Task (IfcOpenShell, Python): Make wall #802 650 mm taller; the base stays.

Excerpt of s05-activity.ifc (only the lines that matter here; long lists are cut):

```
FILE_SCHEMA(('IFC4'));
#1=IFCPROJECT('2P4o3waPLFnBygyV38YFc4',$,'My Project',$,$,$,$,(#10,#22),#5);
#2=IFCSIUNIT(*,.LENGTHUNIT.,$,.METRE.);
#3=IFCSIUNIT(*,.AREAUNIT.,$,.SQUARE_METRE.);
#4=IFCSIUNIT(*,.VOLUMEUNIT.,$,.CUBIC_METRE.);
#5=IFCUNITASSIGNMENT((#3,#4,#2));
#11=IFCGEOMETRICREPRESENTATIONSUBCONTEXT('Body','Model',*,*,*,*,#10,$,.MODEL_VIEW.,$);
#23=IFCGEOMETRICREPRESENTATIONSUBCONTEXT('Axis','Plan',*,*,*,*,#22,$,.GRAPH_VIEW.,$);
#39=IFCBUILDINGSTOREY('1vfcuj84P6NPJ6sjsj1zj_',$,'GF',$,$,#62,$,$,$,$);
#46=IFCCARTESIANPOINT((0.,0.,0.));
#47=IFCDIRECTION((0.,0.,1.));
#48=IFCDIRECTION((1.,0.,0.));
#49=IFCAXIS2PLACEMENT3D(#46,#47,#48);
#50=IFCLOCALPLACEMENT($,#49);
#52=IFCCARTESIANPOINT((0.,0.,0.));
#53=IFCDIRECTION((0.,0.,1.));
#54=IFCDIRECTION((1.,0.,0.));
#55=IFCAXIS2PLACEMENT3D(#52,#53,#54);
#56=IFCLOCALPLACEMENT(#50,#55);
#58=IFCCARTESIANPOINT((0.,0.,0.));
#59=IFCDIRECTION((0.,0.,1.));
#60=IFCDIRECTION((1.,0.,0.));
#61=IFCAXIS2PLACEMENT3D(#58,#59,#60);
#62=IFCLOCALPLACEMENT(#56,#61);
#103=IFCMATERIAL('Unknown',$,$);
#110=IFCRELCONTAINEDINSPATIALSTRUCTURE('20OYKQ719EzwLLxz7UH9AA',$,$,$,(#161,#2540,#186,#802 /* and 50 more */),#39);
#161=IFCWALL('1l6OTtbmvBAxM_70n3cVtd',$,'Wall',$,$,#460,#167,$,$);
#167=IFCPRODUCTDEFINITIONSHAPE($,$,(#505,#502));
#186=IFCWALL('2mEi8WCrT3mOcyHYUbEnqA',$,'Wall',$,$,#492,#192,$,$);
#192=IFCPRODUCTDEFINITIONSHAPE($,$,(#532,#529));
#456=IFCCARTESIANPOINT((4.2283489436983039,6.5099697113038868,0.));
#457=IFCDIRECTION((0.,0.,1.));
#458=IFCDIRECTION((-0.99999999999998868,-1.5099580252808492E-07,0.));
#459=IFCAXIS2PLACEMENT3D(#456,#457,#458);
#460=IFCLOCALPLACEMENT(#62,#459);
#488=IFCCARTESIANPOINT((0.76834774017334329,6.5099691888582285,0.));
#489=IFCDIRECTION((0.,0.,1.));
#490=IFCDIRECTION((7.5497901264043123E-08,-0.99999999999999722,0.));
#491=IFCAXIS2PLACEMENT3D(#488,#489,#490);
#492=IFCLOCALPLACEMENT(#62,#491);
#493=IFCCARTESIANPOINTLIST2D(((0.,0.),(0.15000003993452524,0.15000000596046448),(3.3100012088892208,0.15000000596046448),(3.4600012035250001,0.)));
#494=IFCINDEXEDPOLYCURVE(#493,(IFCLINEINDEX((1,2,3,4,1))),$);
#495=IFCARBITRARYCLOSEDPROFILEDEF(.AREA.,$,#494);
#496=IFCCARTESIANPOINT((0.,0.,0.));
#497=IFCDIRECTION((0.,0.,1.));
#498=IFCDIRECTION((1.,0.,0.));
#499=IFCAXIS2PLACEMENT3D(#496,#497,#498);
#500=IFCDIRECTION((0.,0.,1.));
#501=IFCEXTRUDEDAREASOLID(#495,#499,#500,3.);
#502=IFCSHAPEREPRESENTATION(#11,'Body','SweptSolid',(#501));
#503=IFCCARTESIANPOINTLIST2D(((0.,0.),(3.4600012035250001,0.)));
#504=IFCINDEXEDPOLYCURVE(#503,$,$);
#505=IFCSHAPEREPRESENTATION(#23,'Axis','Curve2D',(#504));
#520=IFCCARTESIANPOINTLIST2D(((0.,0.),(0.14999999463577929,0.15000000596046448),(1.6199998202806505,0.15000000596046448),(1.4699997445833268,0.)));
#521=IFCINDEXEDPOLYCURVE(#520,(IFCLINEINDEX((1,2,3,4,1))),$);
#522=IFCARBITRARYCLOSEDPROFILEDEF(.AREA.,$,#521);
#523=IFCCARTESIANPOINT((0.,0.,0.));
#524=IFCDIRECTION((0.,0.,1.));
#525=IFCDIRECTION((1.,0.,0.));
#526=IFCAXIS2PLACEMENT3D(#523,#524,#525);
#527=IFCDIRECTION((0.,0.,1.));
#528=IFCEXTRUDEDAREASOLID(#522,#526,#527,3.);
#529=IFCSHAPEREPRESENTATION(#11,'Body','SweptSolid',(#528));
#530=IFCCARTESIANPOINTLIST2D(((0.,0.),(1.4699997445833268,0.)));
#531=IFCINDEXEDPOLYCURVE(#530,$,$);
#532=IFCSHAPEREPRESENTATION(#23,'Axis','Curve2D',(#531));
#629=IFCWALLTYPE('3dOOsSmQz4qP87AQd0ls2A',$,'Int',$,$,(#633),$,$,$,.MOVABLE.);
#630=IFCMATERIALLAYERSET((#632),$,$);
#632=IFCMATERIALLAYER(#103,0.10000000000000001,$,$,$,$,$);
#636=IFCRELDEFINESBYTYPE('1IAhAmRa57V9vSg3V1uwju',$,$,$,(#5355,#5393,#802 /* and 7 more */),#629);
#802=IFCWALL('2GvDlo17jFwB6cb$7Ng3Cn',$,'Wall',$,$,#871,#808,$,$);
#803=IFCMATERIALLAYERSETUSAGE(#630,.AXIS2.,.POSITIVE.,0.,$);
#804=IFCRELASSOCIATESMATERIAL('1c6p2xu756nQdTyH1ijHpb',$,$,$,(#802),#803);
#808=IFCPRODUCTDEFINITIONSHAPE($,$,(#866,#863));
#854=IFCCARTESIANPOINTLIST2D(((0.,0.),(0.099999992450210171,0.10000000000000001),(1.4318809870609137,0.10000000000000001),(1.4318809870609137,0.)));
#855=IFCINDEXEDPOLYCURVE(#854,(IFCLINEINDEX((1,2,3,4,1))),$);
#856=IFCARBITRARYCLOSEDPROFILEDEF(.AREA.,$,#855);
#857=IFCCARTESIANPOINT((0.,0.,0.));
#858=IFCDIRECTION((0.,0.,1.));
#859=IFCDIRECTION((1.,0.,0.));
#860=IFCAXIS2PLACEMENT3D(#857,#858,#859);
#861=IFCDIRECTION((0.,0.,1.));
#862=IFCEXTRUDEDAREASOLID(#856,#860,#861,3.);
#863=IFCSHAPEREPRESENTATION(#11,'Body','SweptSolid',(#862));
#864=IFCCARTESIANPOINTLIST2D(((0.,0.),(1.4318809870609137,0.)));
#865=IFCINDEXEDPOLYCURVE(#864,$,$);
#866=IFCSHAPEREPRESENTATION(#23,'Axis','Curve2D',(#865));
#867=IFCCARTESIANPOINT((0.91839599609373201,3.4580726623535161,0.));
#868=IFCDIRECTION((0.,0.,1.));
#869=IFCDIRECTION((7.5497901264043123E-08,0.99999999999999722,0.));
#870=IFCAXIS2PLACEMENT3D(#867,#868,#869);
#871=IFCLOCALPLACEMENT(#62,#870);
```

```python
import ifcopenshell
import ifcopenshell.geom
import ifcopenshell.util.representation
import ifcopenshell.util.shape

model = ifcopenshell.open("s05-activity.ifc")
settings = ifcopenshell.geom.settings()


def volume(element):
    """Net volume in cubic metres, openings subtracted."""
    shape = ifcopenshell.geom.create_shape(settings, element)
    return ifcopenshell.util.shape.get_volume(shape.geometry)


wall = model.by_guid("2GvDlo17jFwB6cb$7Ng3Cn")
before = volume(wall)

body = ifcopenshell.util.representation.get_representation(wall, "Model", "Body")
solid = body.Items[0]
old_height = solid.Depth
solid.Depth += 0.65
after = volume(wall)

print(f"height {old_height:g} -> {solid.Depth:g}, volume {before:.3f} -> {after:.3f} m3")

model.write("s05-activity_v2.ifc")
```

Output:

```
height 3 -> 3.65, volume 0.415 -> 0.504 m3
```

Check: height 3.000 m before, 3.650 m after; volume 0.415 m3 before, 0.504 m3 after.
